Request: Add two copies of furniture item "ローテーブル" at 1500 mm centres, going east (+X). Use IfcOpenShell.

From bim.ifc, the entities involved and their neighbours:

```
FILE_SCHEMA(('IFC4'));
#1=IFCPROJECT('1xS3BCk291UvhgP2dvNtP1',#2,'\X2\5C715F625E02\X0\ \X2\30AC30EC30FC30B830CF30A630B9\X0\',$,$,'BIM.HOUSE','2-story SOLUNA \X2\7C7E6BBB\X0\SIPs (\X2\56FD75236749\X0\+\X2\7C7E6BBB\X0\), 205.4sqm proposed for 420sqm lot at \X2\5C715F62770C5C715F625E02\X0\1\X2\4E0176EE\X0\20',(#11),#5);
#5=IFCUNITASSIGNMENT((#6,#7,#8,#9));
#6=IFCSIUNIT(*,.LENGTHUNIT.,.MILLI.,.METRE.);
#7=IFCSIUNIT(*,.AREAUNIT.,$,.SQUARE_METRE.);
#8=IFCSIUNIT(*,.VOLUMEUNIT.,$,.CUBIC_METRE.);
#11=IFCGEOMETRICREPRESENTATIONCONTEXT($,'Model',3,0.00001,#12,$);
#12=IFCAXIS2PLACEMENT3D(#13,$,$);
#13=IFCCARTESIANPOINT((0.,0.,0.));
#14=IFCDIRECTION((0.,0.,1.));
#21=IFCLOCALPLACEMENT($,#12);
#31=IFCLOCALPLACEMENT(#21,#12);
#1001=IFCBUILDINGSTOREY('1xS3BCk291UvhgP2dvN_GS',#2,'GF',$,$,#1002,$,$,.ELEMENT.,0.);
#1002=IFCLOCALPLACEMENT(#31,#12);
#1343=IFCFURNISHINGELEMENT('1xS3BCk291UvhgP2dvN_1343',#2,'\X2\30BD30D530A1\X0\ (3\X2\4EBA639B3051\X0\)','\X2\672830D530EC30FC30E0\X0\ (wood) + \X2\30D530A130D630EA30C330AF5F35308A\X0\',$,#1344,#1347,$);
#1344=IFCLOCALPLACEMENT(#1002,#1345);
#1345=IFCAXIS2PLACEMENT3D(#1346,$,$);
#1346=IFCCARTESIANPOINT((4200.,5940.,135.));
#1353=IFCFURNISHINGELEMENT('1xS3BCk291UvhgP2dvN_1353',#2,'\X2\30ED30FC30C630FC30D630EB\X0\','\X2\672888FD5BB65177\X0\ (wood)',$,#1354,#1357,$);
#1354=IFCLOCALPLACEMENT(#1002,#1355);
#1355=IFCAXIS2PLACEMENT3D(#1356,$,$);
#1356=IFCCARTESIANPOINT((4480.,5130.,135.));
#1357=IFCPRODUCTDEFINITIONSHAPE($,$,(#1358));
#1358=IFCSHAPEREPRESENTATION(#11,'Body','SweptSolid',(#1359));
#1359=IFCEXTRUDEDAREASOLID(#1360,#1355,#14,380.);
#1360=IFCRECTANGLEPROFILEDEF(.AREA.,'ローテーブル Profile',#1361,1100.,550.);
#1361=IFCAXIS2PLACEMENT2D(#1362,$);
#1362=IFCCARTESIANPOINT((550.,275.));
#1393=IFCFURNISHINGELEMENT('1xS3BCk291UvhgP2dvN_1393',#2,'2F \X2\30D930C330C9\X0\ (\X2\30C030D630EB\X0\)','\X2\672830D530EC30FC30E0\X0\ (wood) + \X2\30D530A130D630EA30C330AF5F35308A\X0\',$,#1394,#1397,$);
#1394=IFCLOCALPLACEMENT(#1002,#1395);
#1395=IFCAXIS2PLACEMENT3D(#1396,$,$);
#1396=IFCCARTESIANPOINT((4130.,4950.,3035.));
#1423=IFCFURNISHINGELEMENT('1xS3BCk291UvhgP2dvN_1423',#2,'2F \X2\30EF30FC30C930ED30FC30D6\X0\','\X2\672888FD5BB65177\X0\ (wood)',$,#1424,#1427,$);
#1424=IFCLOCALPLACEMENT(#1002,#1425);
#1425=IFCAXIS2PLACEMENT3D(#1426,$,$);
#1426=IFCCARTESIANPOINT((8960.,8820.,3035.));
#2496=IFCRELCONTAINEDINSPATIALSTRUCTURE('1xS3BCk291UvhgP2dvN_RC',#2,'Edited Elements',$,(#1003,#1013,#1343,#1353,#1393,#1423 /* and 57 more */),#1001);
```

```python
import numpy as np
import ifcopenshell
import ifcopenshell.api.geometry
import ifcopenshell.api.root
import ifcopenshell.util.element
import ifcopenshell.util.placement
import ifcopenshell.util.unit

model = ifcopenshell.open("bim.ifc")
unit_scale = ifcopenshell.util.unit.calculate_unit_scale(model)


def reuse_history(source, copy):
    """copy_class also copies each property set's owner history, people and application; keep the originals."""
    for rel in copy.IsDefinedBy:
        if rel.is_a("IfcRelDefinesByProperties") and (history := rel.RelatingPropertyDefinition.OwnerHistory):
            rel.RelatingPropertyDefinition.OwnerHistory = source.OwnerHistory
            ifcopenshell.util.element.remove_deep2(model, history)


source = model.by_id(1353)
base = ifcopenshell.util.placement.get_local_placement(source.ObjectPlacement)
step = np.array([1.0, 0.0, 0.0]) * 1.5 / unit_scale

for i in range(1, 3):
    copy = ifcopenshell.api.root.copy_class(model, product=source)
    copy.Representation = ifcopenshell.util.element.copy_deep(
        model, source.Representation, exclude=["IfcGeometricRepresentationContext", "IfcRepresentationMap"]
    )
    reuse_history(source, copy)
    matrix = base.copy()
    matrix[:3, 3] += i * step
    print("added at", matrix[:3, 3].round(3) + 0.0)
    ifcopenshell.api.geometry.edit_object_placement(model, product=copy, matrix=matrix, is_si=False)

model.write("bim-out.ifc")
```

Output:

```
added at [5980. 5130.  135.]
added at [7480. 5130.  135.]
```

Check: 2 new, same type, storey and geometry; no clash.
